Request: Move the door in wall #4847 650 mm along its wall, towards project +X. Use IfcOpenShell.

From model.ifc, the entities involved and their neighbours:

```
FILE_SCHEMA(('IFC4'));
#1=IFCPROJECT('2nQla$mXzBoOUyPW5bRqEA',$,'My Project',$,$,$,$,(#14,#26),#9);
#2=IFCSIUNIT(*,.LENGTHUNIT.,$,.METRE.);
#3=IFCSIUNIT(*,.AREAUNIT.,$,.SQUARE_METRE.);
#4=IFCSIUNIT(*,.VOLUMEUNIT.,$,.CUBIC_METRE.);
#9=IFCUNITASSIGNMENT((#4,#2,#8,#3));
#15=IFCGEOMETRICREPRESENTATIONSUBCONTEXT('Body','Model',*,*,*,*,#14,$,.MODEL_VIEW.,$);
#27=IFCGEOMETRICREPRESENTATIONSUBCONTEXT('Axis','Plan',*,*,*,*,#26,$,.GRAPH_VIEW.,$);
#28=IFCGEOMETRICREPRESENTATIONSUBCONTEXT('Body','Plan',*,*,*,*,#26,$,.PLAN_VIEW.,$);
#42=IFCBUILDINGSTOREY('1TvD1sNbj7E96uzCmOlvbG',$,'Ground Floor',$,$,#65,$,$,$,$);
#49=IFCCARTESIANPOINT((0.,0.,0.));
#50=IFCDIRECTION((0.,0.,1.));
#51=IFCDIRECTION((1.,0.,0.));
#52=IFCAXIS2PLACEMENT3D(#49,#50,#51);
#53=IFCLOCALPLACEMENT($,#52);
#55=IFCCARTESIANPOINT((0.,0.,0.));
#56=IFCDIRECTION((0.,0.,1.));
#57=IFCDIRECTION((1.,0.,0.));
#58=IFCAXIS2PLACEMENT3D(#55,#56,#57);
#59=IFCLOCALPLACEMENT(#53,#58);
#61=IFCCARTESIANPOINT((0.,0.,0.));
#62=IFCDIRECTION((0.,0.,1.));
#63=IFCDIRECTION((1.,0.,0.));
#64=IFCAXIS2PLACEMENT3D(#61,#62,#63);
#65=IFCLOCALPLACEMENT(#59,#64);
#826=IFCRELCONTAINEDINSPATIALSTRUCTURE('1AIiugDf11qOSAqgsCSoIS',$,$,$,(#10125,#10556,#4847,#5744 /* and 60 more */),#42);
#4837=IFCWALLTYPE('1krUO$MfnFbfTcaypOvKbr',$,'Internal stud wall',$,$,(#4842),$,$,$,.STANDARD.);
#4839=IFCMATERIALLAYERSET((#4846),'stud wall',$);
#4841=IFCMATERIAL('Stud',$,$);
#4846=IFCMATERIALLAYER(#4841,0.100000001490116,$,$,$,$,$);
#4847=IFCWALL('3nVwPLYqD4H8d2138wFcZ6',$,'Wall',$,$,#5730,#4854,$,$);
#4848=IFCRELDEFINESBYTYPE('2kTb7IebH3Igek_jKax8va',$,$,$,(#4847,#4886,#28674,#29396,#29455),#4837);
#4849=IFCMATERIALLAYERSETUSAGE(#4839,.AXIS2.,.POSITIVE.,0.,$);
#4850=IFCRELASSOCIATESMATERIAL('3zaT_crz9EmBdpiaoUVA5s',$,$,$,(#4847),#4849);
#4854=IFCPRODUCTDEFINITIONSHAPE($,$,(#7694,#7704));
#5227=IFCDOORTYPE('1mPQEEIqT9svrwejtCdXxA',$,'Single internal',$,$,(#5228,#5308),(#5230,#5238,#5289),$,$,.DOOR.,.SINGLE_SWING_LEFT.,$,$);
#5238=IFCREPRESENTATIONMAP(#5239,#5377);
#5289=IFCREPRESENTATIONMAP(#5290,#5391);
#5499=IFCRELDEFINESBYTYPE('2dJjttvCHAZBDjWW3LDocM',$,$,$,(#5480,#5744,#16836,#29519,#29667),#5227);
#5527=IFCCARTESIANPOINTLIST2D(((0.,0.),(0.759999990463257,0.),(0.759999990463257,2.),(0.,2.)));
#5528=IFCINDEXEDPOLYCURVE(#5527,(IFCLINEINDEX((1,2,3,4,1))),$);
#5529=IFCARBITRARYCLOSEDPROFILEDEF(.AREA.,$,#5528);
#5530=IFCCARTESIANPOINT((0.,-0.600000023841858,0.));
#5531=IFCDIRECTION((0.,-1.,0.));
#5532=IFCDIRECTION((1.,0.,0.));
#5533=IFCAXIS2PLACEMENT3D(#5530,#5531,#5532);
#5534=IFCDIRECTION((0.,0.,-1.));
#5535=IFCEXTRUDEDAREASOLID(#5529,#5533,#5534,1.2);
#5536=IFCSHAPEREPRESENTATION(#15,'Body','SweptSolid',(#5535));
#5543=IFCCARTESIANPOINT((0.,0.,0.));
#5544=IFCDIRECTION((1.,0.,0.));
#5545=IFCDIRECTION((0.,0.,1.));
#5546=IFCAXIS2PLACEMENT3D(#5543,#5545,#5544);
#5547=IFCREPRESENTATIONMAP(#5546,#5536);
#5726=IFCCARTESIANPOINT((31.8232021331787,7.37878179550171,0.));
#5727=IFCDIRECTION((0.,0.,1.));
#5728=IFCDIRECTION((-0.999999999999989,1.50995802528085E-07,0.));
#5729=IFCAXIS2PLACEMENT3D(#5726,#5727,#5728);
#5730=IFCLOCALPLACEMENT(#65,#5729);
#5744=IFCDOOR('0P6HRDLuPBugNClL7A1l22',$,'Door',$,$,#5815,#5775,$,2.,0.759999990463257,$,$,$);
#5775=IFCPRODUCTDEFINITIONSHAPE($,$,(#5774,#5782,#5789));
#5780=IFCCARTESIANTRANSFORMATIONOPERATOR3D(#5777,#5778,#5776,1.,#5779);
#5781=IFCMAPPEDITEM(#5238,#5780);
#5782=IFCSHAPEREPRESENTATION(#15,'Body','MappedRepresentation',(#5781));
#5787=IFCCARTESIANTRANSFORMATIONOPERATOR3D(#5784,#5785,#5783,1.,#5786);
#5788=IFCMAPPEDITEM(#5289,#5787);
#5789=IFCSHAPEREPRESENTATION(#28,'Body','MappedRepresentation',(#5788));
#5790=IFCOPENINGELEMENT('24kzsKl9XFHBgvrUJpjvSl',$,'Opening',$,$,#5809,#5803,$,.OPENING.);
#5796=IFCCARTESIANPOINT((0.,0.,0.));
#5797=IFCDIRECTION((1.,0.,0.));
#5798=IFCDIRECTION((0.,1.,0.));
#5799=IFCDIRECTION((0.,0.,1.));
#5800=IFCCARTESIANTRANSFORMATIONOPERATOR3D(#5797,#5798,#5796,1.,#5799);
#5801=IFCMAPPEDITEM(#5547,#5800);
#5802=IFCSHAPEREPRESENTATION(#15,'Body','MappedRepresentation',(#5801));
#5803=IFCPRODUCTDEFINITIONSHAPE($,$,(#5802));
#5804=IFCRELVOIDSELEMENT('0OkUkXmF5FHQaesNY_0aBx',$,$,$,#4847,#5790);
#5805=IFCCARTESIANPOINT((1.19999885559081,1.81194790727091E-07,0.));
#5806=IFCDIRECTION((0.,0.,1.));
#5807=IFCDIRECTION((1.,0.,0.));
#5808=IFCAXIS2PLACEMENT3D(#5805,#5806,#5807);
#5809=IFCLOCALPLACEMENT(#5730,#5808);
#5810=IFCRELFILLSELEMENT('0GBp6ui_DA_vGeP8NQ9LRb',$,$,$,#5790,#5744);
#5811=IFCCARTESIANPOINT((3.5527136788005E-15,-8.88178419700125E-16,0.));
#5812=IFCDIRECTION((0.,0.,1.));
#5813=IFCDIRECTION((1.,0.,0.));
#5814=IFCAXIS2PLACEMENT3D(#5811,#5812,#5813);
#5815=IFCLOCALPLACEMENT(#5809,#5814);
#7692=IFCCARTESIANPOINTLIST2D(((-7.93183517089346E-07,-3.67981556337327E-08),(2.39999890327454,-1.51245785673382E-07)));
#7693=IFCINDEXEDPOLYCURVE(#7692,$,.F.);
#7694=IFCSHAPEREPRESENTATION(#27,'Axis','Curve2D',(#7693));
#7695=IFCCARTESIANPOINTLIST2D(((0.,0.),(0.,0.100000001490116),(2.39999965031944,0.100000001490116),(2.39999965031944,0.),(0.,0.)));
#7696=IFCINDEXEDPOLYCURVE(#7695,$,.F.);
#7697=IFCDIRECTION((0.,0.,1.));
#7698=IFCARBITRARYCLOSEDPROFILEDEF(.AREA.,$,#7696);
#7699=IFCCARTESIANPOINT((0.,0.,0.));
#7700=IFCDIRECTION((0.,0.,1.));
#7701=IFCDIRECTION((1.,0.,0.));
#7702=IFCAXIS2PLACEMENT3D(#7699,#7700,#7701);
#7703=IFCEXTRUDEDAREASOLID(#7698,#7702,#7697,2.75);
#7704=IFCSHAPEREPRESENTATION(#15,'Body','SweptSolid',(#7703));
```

```python
import ifcopenshell
import ifcopenshell.api.geometry
import ifcopenshell.util.placement
import ifcopenshell.util.unit

model = ifcopenshell.open("model.ifc")
unit_scale = ifcopenshell.util.unit.calculate_unit_scale(model)

door = model.by_guid("0P6HRDLuPBugNClL7A1l22")
opening = door.FillsVoids[0].RelatingOpeningElement
wall = opening.VoidsElements[0].RelatingBuildingElement

wall_matrix = ifcopenshell.util.placement.get_local_placement(wall.ObjectPlacement)
shift = wall_matrix[:3, 0] * -0.65 / unit_scale
before = ifcopenshell.util.placement.get_local_placement(door.ObjectPlacement)[:3, 3].copy()

# The door is placed relative to its opening, so it follows when the opening moves.
matrix = ifcopenshell.util.placement.get_local_placement(opening.ObjectPlacement)
matrix[:3, 3] += shift
ifcopenshell.api.geometry.edit_object_placement(
    model, product=opening, matrix=matrix, is_si=False, should_transform_children=True
)

after = ifcopenshell.util.placement.get_local_placement(door.ObjectPlacement)[:3, 3]
print("door moved by", (after - before).round(3) + 0.0)

model.write("model-out.ifc")
```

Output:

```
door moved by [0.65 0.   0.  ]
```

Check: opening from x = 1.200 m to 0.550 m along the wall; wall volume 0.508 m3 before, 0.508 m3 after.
